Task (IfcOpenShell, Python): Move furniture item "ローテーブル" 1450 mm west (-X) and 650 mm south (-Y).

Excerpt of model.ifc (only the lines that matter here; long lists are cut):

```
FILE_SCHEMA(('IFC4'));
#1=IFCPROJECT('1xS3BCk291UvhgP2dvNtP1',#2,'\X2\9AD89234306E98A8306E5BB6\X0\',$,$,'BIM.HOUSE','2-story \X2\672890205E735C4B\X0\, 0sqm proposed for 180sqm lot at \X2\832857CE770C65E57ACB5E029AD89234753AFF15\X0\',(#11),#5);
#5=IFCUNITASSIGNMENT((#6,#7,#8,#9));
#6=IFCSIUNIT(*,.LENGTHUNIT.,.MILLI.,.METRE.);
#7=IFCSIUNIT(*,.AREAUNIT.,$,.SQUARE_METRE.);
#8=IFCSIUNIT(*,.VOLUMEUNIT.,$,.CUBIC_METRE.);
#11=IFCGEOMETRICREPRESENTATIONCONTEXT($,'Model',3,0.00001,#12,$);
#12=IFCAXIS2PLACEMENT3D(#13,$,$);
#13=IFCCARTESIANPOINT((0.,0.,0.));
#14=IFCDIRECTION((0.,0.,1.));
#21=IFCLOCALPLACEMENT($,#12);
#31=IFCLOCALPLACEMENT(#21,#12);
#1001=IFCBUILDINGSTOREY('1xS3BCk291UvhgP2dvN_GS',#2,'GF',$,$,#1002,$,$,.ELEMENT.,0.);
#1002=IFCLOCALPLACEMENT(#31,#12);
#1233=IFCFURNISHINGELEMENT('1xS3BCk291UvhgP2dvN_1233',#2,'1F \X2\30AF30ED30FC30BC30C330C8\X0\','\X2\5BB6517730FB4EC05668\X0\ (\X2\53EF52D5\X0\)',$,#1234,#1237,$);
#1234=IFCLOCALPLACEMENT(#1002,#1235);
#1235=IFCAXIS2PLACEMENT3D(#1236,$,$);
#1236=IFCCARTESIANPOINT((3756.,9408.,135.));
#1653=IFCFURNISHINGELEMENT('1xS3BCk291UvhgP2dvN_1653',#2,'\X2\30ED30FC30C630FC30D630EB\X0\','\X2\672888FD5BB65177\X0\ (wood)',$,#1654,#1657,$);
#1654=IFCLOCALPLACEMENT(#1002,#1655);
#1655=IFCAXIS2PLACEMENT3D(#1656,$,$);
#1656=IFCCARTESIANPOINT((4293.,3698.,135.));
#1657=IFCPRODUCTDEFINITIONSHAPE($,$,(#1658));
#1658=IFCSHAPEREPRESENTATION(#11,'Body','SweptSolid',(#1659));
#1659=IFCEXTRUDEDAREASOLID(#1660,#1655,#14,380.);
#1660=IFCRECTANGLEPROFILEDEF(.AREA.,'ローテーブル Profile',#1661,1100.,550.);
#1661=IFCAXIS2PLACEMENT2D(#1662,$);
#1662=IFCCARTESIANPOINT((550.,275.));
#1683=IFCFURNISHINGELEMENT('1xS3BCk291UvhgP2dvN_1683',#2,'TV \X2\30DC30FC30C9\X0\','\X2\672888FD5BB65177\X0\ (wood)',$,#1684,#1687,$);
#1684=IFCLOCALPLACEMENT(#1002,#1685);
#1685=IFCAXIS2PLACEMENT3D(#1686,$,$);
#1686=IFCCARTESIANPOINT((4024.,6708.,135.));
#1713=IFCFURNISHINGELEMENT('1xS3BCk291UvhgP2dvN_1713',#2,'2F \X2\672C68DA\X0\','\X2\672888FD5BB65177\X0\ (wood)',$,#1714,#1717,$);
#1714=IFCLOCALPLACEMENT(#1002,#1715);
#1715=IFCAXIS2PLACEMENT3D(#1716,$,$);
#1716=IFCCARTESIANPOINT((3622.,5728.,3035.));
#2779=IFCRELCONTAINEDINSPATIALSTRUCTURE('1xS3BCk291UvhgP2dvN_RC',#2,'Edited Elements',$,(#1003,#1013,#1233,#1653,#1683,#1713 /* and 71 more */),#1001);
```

```python
import ifcopenshell
import ifcopenshell.api.geometry
import ifcopenshell.util.placement
import ifcopenshell.util.unit

model = ifcopenshell.open("model.ifc")
unit_scale = ifcopenshell.util.unit.calculate_unit_scale(model)

item = model.by_id(1653)
matrix = ifcopenshell.util.placement.get_local_placement(item.ObjectPlacement)
matrix[0, 3] -= 1.45 / unit_scale
matrix[1, 3] -= 0.65 / unit_scale
ifcopenshell.api.geometry.edit_object_placement(model, product=item, matrix=matrix, is_si=False)

print(ifcopenshell.util.placement.get_local_placement(item.ObjectPlacement).round(3) + 0.0)

model.write("model_v2.ifc")
```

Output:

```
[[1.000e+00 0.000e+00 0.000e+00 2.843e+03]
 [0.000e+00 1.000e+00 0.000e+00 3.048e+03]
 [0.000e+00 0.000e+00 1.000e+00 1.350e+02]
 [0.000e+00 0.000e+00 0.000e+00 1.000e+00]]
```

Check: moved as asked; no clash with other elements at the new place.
